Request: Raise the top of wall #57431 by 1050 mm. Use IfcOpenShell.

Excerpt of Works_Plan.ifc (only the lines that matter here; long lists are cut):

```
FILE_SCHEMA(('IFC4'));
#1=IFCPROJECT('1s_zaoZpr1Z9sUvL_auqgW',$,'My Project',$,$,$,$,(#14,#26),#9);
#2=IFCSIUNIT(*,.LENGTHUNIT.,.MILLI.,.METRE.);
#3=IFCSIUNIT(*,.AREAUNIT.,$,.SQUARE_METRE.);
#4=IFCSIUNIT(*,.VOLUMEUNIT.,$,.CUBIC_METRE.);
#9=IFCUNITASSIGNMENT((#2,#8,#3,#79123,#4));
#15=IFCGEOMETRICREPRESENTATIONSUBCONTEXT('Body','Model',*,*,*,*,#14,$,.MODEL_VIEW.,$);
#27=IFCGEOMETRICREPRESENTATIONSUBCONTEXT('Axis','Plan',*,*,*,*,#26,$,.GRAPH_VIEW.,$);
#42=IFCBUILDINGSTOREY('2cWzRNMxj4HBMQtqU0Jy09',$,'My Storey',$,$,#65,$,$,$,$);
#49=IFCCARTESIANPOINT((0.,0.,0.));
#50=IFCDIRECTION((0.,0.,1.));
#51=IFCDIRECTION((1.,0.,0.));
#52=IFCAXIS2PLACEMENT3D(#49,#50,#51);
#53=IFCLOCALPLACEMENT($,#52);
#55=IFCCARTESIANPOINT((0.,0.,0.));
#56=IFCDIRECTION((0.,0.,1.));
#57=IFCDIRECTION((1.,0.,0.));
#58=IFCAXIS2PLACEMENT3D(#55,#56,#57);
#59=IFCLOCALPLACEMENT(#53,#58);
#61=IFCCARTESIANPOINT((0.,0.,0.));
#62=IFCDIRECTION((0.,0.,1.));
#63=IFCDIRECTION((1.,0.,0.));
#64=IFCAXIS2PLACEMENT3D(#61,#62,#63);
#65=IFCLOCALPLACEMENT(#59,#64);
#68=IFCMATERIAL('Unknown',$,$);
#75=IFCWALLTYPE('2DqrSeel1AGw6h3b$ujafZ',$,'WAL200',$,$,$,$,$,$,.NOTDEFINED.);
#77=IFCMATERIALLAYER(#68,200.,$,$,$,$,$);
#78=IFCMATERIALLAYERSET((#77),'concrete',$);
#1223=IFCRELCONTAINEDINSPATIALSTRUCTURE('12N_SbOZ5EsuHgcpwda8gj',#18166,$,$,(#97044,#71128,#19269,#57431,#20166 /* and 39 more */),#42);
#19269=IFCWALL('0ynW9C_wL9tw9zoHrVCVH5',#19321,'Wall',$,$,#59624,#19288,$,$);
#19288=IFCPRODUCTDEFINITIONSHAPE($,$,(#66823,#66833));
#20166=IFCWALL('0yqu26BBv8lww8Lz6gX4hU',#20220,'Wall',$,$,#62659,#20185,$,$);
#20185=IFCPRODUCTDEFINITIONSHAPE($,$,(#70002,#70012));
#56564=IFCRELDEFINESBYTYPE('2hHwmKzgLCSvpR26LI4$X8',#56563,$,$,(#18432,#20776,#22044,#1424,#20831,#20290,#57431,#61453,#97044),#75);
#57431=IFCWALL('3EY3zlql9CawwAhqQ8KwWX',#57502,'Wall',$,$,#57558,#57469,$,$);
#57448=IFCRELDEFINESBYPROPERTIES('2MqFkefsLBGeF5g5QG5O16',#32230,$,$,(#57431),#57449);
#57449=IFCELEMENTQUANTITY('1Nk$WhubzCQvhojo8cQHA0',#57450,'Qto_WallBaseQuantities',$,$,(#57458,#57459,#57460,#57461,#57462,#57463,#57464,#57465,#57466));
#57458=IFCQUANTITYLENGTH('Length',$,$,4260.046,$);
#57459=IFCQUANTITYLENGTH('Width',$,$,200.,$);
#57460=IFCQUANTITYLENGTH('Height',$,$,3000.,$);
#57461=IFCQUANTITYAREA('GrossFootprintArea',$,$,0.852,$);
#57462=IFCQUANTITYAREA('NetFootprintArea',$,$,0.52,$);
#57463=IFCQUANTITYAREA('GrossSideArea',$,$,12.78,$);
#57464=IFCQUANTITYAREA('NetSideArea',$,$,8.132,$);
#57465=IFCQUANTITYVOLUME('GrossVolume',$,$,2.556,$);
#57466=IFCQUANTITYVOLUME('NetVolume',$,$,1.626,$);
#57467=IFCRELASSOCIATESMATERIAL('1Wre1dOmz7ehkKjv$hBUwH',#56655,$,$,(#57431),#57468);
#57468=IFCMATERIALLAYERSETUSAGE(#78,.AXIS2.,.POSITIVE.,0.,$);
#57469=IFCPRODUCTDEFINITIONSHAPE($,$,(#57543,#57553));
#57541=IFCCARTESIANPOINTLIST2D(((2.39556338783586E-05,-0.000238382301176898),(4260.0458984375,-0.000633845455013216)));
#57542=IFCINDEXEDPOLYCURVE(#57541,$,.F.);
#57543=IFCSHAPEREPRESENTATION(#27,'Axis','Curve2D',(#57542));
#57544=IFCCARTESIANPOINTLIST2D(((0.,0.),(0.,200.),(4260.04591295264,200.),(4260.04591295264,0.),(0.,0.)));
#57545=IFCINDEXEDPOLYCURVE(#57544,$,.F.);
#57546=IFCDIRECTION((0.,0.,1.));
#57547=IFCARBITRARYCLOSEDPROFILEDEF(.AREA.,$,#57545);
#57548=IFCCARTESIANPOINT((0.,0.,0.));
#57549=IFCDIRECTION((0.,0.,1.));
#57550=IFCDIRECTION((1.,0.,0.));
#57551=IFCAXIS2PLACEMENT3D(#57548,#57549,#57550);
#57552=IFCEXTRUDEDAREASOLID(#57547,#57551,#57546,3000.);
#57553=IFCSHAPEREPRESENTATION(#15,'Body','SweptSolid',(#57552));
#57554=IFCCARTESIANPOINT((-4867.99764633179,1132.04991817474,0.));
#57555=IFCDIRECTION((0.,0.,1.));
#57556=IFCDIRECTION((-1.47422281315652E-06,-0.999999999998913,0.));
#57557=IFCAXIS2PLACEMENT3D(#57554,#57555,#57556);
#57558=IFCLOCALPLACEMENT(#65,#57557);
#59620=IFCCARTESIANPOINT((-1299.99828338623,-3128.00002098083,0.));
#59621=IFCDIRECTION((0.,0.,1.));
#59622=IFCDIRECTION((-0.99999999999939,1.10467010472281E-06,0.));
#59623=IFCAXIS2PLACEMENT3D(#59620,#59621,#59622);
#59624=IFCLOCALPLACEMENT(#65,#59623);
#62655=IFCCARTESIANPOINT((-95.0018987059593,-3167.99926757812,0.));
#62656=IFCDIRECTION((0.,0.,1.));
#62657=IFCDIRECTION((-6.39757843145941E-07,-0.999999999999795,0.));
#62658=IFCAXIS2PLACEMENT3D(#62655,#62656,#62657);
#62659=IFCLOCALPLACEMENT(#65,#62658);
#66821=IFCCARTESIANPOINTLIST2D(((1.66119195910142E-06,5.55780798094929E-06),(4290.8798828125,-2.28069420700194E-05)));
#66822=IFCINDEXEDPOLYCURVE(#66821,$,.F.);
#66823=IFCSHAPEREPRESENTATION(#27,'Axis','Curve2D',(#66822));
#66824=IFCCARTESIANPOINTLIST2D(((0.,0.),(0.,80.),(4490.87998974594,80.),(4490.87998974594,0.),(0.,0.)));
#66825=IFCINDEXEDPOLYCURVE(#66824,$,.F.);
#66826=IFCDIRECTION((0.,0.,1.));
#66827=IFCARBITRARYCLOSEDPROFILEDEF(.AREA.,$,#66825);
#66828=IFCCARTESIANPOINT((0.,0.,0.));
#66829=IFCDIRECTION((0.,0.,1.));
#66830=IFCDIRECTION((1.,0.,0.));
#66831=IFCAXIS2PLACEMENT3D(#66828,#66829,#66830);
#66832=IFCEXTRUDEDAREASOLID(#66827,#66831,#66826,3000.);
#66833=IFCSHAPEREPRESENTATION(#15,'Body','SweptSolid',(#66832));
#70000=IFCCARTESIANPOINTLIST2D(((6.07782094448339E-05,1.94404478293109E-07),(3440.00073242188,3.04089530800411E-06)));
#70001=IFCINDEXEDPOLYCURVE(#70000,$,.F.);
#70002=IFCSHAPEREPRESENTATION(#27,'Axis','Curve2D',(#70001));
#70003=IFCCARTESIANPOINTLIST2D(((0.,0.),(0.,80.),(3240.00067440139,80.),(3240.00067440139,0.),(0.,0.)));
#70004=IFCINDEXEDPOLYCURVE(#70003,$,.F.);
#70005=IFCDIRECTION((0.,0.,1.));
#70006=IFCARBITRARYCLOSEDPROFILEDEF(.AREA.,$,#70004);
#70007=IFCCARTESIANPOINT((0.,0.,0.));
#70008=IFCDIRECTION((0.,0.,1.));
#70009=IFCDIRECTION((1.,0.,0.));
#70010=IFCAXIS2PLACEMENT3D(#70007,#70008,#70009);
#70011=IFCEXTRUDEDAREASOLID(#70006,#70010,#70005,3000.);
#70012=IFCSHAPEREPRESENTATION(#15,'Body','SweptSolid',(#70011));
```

```python
import ifcopenshell
import ifcopenshell.api.pset
import ifcopenshell.geom
import ifcopenshell.util.element
import ifcopenshell.util.representation
import ifcopenshell.util.shape
import ifcopenshell.util.unit

model = ifcopenshell.open("Works_Plan.ifc")
unit_scale = ifcopenshell.util.unit.calculate_unit_scale(model)
area_scale = ifcopenshell.util.unit.calculate_unit_scale(model, "AREAUNIT")
volume_scale = ifcopenshell.util.unit.calculate_unit_scale(model, "VOLUMEUNIT")
settings = ifcopenshell.geom.settings()


def volume(element):
    """Net volume in cubic metres, openings subtracted."""
    shape = ifcopenshell.geom.create_shape(settings, element)
    return ifcopenshell.util.shape.get_volume(shape.geometry)


wall = model.by_guid("3EY3zlql9CawwAhqQ8KwWX")
before = volume(wall)

body = ifcopenshell.util.representation.get_representation(wall, "Model", "Body")
solid = body.Items[0]
old_height = solid.Depth
solid.Depth += 1050.0
after = volume(wall)
thickness = 0.2  # wall thickness in metres

# Update the stored height, areas and volumes.
qto = model.by_id(ifcopenshell.util.element.get_pset(wall, "Qto_WallBaseQuantities", should_inherit=False)["id"])
ifcopenshell.api.pset.edit_qto(model, qto=qto, properties={
    "Height": solid.Depth,
    "GrossSideArea": ifcopenshell.util.element.get_pset(wall, "Qto_WallBaseQuantities", "GrossSideArea") * solid.Depth / old_height,
    "NetSideArea": after / thickness / area_scale,
    "GrossVolume": ifcopenshell.util.element.get_pset(wall, "Qto_WallBaseQuantities", "GrossVolume") * solid.Depth / old_height,
    "NetVolume": after / volume_scale,
})

print(f"height {old_height:g} -> {solid.Depth:g}, volume {before:.3f} -> {after:.3f} m3")

model.write("Works_Plan-out.ifc")
```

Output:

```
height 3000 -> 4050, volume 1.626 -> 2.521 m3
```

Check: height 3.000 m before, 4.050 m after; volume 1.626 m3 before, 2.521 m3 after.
